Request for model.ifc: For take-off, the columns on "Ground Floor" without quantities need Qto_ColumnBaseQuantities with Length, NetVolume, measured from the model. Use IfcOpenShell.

First a look at what the model holds.

```python
import ifcopenshell
import ifcopenshell.util.element
import ifcopenshell.util.unit

model = ifcopenshell.open("model.ifc")
print(model.schema)
for unit_type in ("LENGTHUNIT", "AREAUNIT", "VOLUMEUNIT"):
    print(unit_type, ifcopenshell.util.unit.calculate_unit_scale(model, unit_type))
storey = next(s for s in model.by_type("IfcBuildingStorey") if s.Name == "Ground Floor")
columns = [e for e in ifcopenshell.util.element.get_decomposition(storey) if e.is_a("IfcColumn")]
for e in sorted(columns, key=lambda e: e.id()):
    print(e.id(), e.is_a(), e.Name, list(ifcopenshell.util.element.get_psets(e, qtos_only=True)), sep=" | ")
```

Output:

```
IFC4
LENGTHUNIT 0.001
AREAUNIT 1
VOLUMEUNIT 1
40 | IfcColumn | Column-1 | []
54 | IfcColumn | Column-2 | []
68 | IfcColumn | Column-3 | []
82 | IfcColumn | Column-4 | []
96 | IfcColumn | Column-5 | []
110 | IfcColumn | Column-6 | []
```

```python
import ifcopenshell
import ifcopenshell.api.pset
import ifcopenshell.geom
import ifcopenshell.util.element
import ifcopenshell.util.shape
import ifcopenshell.util.unit

model = ifcopenshell.open("model.ifc")
unit_scale = ifcopenshell.util.unit.calculate_unit_scale(model)
volume_scale = ifcopenshell.util.unit.calculate_unit_scale(model, "VOLUMEUNIT")
settings = ifcopenshell.geom.settings()

storey = next(s for s in model.by_type("IfcBuildingStorey") if s.Name == "Ground Floor")
columns = [e for e in ifcopenshell.util.element.get_decomposition(storey) if e.is_a("IfcColumn")]

for e in sorted(columns, key=lambda e: e.id()):
    if ifcopenshell.util.element.get_psets(e, qtos_only=True, should_inherit=False):
        continue
    # Geometry comes back in metres, in the element's own axes.
    shape = ifcopenshell.geom.create_shape(settings, e)
    values = {
        "Length": ifcopenshell.util.shape.get_z(shape.geometry) / unit_scale,
        "NetVolume": ifcopenshell.util.shape.get_volume(shape.geometry) / volume_scale,
    }
    qto = ifcopenshell.api.pset.add_qto(model, product=e, name="Qto_ColumnBaseQuantities")
    ifcopenshell.api.pset.edit_qto(model, qto=qto, properties=values)
    print(e.id(), {k: round(v, 3) for k, v in values.items()})

model.write("model_updated.ifc")
```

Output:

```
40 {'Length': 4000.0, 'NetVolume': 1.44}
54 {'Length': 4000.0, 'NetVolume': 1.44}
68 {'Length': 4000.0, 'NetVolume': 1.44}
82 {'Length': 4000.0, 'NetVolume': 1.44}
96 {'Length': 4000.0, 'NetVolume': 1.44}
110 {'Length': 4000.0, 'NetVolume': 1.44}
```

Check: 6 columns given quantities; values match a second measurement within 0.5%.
